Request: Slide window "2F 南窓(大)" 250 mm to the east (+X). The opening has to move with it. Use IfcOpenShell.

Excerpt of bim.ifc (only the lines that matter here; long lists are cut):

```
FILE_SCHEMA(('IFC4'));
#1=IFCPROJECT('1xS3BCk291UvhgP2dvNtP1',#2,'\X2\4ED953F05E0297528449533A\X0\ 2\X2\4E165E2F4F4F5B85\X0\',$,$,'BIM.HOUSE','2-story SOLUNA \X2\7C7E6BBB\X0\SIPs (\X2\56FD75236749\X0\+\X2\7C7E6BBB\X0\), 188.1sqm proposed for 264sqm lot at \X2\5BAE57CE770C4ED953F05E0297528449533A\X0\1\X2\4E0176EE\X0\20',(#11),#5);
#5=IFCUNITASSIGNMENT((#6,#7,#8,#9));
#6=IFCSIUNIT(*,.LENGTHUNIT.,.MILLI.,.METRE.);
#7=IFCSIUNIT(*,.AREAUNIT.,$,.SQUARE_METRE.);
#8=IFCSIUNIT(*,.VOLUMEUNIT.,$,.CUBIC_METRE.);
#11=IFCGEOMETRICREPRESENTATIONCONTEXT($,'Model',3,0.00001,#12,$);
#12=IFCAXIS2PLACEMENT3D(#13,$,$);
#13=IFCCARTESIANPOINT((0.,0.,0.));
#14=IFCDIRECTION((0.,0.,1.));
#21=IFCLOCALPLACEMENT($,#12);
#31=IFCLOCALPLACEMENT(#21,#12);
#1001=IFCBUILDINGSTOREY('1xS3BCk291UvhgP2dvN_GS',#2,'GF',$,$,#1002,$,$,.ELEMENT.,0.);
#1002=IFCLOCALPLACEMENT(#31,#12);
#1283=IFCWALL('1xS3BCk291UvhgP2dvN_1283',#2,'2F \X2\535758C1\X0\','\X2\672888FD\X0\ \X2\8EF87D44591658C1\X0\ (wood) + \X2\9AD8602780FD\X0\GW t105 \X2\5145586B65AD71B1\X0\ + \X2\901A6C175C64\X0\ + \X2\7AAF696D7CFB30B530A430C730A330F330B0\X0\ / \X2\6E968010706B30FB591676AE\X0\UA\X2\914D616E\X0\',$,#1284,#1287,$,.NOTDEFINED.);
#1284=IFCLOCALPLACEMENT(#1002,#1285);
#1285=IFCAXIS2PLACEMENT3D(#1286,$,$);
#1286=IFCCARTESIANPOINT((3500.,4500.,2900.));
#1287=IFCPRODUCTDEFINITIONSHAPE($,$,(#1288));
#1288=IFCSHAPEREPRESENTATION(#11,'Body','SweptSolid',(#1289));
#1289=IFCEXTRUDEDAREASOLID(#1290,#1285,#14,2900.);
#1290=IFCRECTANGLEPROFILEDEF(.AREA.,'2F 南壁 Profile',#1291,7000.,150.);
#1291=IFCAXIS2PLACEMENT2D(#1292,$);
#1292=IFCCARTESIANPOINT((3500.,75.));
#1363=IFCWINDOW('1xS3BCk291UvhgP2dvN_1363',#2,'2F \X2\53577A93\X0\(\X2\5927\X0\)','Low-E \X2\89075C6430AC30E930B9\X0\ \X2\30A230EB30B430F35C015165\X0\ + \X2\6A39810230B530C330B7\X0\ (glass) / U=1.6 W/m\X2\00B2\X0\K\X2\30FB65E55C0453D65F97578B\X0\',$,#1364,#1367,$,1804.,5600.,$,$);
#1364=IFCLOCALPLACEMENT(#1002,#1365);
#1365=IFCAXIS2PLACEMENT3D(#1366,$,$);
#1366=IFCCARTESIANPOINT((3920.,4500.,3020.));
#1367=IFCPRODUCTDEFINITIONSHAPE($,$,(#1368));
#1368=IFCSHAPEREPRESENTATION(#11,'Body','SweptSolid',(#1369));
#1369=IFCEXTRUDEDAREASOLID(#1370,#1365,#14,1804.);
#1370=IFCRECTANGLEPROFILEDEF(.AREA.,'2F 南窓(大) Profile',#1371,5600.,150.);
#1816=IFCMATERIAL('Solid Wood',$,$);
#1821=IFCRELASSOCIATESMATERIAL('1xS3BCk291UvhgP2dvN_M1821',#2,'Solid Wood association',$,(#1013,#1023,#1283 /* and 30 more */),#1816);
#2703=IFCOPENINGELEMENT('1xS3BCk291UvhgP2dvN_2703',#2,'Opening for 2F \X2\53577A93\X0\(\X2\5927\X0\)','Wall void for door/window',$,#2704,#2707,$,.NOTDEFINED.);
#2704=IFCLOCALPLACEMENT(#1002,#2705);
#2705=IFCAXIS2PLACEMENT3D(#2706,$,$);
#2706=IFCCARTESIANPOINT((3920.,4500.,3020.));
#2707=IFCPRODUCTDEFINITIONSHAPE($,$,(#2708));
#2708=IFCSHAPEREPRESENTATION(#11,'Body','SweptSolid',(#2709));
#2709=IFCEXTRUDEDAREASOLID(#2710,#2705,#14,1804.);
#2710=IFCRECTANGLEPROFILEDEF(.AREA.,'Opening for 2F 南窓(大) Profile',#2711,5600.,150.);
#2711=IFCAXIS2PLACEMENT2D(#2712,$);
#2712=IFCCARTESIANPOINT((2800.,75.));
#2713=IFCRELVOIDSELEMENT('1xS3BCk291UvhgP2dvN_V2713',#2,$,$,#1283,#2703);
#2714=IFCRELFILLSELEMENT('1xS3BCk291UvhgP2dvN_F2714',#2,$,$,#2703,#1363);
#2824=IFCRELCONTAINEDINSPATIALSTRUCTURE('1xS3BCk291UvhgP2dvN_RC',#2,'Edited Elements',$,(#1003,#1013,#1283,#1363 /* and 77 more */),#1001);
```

```python
import ifcopenshell
import ifcopenshell.api.geometry
import ifcopenshell.util.placement
import ifcopenshell.util.unit

model = ifcopenshell.open("bim.ifc")
unit_scale = ifcopenshell.util.unit.calculate_unit_scale(model)

window = model.by_id(1363)
opening = window.FillsVoids[0].RelatingOpeningElement
wall = opening.VoidsElements[0].RelatingBuildingElement

wall_matrix = ifcopenshell.util.placement.get_local_placement(wall.ObjectPlacement)
shift = wall_matrix[:3, 0] * 0.25 / unit_scale
before = ifcopenshell.util.placement.get_local_placement(window.ObjectPlacement)[:3, 3].copy()

# The window is not placed relative to its opening, so move both.
for product in (opening, window):
    matrix = ifcopenshell.util.placement.get_local_placement(product.ObjectPlacement)
    matrix[:3, 3] += shift
    ifcopenshell.api.geometry.edit_object_placement(model, product=product, matrix=matrix, is_si=False)

after = ifcopenshell.util.placement.get_local_placement(window.ObjectPlacement)[:3, 3]
print("window moved by", (after - before).round(3) + 0.0)

model.write("bim-out.ifc")
```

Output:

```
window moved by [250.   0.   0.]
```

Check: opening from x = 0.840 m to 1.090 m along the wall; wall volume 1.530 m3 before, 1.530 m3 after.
